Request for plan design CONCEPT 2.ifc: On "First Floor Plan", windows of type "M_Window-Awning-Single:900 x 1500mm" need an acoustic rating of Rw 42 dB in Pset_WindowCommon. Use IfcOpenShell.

First a look at what the model holds.

```python
import ifcopenshell
import ifcopenshell.util.element

model = ifcopenshell.open("plan design CONCEPT 2.ifc")
print(model.schema)
storey = next(s for s in model.by_type("IfcBuildingStorey") if s.Name == "First Floor Plan")
windows = [e for e in ifcopenshell.util.element.get_decomposition(storey) if e.is_a("IfcWindow")]
seen = {}
for e in windows:
    element_type = ifcopenshell.util.element.get_type(e)
    key = (element_type.Name if element_type != e and element_type else None, ifcopenshell.util.element.get_pset(e, "Pset_WindowCommon", "AcousticRating"))
    seen[key] = seen.get(key, 0) + 1
for (name, value), count in sorted(seen.items(), key=str):
    print(count, "x", name, "|", value)
```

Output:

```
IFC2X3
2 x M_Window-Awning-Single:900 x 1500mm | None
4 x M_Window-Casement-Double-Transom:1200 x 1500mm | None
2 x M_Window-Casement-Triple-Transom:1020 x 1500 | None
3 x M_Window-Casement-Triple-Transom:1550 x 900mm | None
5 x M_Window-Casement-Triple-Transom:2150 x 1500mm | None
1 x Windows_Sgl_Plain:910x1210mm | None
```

```python
import ifcopenshell
import ifcopenshell.api.pset
import ifcopenshell.util.element

model = ifcopenshell.open("plan design CONCEPT 2.ifc")

storey = next(s for s in model.by_type("IfcBuildingStorey") if s.Name == "First Floor Plan")
windows = [e for e in ifcopenshell.util.element.get_decomposition(storey) if e.is_a("IfcWindow")]

count = 0
for e in windows:
    element_type = ifcopenshell.util.element.get_type(e)
    if element_type in (None, e) or element_type.Name != "M_Window-Awning-Single:900 x 1500mm":
        continue
    # add_pset returns the element's existing set when there is one.
    pset = ifcopenshell.api.pset.add_pset(model, product=e, name="Pset_WindowCommon")
    ifcopenshell.api.pset.edit_pset(model, pset=pset, properties={"AcousticRating": "Rw 42 dB"})
    count += 1

print(count, "windows updated")

model.write("plan design CONCEPT 2_rev.ifc")
```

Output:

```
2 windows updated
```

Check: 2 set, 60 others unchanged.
